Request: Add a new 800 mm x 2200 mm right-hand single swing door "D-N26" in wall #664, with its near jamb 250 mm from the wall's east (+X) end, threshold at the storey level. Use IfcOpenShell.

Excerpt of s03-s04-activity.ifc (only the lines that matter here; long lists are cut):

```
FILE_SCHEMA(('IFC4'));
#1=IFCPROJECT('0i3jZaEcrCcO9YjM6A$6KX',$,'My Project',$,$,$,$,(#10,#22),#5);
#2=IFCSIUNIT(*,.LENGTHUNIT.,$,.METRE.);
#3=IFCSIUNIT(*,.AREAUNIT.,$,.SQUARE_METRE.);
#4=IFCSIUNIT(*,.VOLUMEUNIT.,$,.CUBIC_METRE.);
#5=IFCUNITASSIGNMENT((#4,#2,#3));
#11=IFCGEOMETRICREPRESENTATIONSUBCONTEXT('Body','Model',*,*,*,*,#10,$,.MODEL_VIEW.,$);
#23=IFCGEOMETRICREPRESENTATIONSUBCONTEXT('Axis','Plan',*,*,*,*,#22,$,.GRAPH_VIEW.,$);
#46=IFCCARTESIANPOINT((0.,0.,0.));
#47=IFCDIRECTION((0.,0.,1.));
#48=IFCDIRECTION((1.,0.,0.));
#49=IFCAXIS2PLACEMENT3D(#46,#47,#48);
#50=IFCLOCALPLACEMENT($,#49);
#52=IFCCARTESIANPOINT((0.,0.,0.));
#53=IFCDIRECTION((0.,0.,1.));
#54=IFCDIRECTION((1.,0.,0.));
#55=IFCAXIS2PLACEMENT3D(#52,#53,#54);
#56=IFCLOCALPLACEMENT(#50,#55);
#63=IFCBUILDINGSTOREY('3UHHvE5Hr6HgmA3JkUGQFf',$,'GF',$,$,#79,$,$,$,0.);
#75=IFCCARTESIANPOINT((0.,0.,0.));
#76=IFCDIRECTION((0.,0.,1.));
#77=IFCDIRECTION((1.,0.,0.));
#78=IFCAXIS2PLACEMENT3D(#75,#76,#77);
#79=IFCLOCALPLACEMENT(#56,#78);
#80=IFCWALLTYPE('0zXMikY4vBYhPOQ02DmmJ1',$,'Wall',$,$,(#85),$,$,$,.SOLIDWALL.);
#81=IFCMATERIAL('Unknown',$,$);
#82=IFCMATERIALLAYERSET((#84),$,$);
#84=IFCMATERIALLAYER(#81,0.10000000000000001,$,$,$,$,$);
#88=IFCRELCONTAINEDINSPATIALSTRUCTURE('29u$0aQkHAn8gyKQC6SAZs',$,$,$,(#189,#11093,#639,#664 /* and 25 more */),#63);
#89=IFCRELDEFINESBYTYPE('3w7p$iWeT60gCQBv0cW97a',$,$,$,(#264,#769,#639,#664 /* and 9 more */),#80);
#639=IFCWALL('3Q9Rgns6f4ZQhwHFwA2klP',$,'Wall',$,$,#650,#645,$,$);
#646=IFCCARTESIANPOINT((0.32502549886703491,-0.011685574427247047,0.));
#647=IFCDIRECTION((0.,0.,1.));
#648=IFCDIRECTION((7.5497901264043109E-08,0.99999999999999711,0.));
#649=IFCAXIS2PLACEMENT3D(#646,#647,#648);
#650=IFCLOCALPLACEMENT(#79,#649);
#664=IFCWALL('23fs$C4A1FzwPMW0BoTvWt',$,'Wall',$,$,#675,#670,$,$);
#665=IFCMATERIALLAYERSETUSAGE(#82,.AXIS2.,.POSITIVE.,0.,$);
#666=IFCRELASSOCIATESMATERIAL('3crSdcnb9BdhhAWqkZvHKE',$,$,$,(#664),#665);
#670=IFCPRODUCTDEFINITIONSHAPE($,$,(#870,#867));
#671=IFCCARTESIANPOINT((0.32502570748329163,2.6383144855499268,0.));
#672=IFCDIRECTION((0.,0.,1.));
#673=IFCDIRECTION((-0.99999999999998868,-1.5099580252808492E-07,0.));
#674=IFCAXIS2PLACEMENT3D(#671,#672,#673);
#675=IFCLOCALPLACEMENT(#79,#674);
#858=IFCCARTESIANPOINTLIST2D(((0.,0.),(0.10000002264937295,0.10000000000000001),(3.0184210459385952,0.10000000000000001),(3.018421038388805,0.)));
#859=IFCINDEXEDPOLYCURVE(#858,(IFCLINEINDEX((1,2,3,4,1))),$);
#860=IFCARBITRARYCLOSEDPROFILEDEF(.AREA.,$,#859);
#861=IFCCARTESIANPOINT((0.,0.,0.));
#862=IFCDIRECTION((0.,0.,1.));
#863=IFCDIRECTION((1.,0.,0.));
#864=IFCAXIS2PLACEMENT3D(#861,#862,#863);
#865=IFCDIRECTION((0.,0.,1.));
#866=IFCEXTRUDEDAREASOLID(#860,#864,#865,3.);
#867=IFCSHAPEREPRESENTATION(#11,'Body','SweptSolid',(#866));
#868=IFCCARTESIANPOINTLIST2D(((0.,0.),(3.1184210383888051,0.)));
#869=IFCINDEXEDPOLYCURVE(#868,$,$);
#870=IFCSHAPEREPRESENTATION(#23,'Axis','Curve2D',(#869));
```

```python
import numpy as np
import ifcopenshell
import ifcopenshell.api.feature
import ifcopenshell.api.geometry
import ifcopenshell.api.root
import ifcopenshell.api.spatial
import ifcopenshell.geom
import ifcopenshell.util.element
import ifcopenshell.util.placement
import ifcopenshell.util.representation
import ifcopenshell.util.shape
import ifcopenshell.util.unit

model = ifcopenshell.open("s03-s04-activity.ifc")
unit_scale = ifcopenshell.util.unit.calculate_unit_scale(model)
settings = ifcopenshell.geom.settings()


def volume(element):
    """Net volume in cubic metres, openings subtracted."""
    shape = ifcopenshell.geom.create_shape(settings, element)
    return ifcopenshell.util.shape.get_volume(shape.geometry)


wall = model.by_id(664)
storey = ifcopenshell.util.element.get_container(wall, ifc_class="IfcBuildingStorey")
context = ifcopenshell.util.representation.get_context(model, "Model", "Body", "MODEL_VIEW")
before = volume(wall)

width, height, from_end, sill = 0.8, 2.2, 0.25, 0.0  # metres

# The wall runs along its own X axis, and the end named is its -X end.
wall_shape = ifcopenshell.geom.create_shape(settings, wall)
x, y, z = ifcopenshell.util.shape.get_vertices(wall_shape.geometry).T
start = x.min() + from_end
face, thickness = float(y.min()), float(y.max() - y.min())
wall_matrix = ifcopenshell.util.placement.get_local_placement(wall.ObjectPlacement)
level = ifcopenshell.util.placement.get_local_placement(storey.ObjectPlacement)[2, 3]


def in_wall(x, y):
    """Placement at x, y metres in the wall's axes, at sill height."""
    matrix = wall_matrix.copy()
    matrix[:, 3] = wall_matrix @ np.array([x / unit_scale, y / unit_scale, 0.0, 1.0])
    matrix[2, 3] = level + sill / unit_scale
    return matrix


# Opening: a box that overshoots both wall faces by 50 mm.
opening = ifcopenshell.api.root.create_entity(model, ifc_class="IfcOpeningElement", predefined_type="OPENING")
box = ifcopenshell.api.geometry.add_wall_representation(
    model, context=context, length=width, height=height, thickness=thickness + 0.1
)
ifcopenshell.api.geometry.assign_representation(model, product=opening, representation=box)
ifcopenshell.api.geometry.edit_object_placement(model, product=opening, matrix=in_wall(start, face - 0.05), is_si=False)
ifcopenshell.api.feature.add_feature(model, feature=opening, element=wall)

door = ifcopenshell.api.root.create_entity(model, ifc_class="IfcDoor", name="D-N26", predefined_type="DOOR")
door.OverallWidth, door.OverallHeight = width / unit_scale, height / unit_scale
door.OperationType = "SINGLE_SWING_RIGHT"
body = ifcopenshell.api.geometry.add_door_representation(
    model,
    context=context,
    overall_width=door.OverallWidth,
    overall_height=door.OverallHeight,
    operation_type="SINGLE_SWING_RIGHT",
    lining_properties={"LiningDepth": thickness / unit_scale, "ThresholdDepth": thickness / unit_scale},
)
ifcopenshell.api.geometry.assign_representation(model, product=door, representation=body)
ifcopenshell.api.spatial.assign_container(model, products=[door], relating_structure=storey)
ifcopenshell.api.feature.add_filling(model, opening=opening, element=door)

# The lining spans the wall, so the door starts at the wall face.
ifcopenshell.api.geometry.edit_object_placement(model, product=door, matrix=in_wall(start, face), is_si=False)

after = volume(wall)

print(f"wall volume {before:.3f} -> {after:.3f} m3")

model.write("s03-s04-activity_updated.ifc")
```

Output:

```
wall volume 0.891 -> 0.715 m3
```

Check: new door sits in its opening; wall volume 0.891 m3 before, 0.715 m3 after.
